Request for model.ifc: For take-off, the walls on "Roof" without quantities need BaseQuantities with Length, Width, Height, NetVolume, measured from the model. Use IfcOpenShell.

First a look at what the model holds.

```python
import ifcopenshell
import ifcopenshell.util.element
import ifcopenshell.util.unit

model = ifcopenshell.open("model.ifc")
print(model.schema)
for unit_type in ("LENGTHUNIT", "AREAUNIT", "VOLUMEUNIT"):
    print(unit_type, ifcopenshell.util.unit.calculate_unit_scale(model, unit_type))
storey = next(s for s in model.by_type("IfcBuildingStorey") if s.Name == "Roof")
walls = [e for e in ifcopenshell.util.element.get_decomposition(storey) if e.is_a("IfcWall")]
for e in sorted(walls, key=lambda e: e.id()):
    print(e.id(), e.is_a(), e.Name, list(ifcopenshell.util.element.get_psets(e, qtos_only=True)), sep=" | ")
```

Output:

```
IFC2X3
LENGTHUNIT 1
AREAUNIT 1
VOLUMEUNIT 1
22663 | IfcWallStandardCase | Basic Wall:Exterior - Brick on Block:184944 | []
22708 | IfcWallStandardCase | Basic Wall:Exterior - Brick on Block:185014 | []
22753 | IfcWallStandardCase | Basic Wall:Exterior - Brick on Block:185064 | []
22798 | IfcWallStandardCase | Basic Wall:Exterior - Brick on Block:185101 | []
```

```python
import ifcopenshell
import ifcopenshell.api.pset
import ifcopenshell.geom
import ifcopenshell.util.element
import ifcopenshell.util.shape
import ifcopenshell.util.unit

model = ifcopenshell.open("model.ifc")
unit_scale = ifcopenshell.util.unit.calculate_unit_scale(model)
volume_scale = ifcopenshell.util.unit.calculate_unit_scale(model, "VOLUMEUNIT")
settings = ifcopenshell.geom.settings()

storey = next(s for s in model.by_type("IfcBuildingStorey") if s.Name == "Roof")
walls = [e for e in ifcopenshell.util.element.get_decomposition(storey) if e.is_a("IfcWall")]

for e in sorted(walls, key=lambda e: e.id()):
    if ifcopenshell.util.element.get_psets(e, qtos_only=True, should_inherit=False):
        continue
    # Geometry comes back in metres, in the element's own axes.
    shape = ifcopenshell.geom.create_shape(settings, e)
    values = {
        "Length": ifcopenshell.util.shape.get_x(shape.geometry) / unit_scale,
        "Width": ifcopenshell.util.shape.get_y(shape.geometry) / unit_scale,
        "Height": ifcopenshell.util.shape.get_z(shape.geometry) / unit_scale,
        "NetVolume": ifcopenshell.util.shape.get_volume(shape.geometry) / volume_scale,
    }
    qto = ifcopenshell.api.pset.add_qto(model, product=e, name="BaseQuantities")
    ifcopenshell.api.pset.edit_qto(model, qto=qto, properties=values)
    print(e.id(), {k: round(v, 3) for k, v in values.items()})

model.write("model_edited.ifc")
```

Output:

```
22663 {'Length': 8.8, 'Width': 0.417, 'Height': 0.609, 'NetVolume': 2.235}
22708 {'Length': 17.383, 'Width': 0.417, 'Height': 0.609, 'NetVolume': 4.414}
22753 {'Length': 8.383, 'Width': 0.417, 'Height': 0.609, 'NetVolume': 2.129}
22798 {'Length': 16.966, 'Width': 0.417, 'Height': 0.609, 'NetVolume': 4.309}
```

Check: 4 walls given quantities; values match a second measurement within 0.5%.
